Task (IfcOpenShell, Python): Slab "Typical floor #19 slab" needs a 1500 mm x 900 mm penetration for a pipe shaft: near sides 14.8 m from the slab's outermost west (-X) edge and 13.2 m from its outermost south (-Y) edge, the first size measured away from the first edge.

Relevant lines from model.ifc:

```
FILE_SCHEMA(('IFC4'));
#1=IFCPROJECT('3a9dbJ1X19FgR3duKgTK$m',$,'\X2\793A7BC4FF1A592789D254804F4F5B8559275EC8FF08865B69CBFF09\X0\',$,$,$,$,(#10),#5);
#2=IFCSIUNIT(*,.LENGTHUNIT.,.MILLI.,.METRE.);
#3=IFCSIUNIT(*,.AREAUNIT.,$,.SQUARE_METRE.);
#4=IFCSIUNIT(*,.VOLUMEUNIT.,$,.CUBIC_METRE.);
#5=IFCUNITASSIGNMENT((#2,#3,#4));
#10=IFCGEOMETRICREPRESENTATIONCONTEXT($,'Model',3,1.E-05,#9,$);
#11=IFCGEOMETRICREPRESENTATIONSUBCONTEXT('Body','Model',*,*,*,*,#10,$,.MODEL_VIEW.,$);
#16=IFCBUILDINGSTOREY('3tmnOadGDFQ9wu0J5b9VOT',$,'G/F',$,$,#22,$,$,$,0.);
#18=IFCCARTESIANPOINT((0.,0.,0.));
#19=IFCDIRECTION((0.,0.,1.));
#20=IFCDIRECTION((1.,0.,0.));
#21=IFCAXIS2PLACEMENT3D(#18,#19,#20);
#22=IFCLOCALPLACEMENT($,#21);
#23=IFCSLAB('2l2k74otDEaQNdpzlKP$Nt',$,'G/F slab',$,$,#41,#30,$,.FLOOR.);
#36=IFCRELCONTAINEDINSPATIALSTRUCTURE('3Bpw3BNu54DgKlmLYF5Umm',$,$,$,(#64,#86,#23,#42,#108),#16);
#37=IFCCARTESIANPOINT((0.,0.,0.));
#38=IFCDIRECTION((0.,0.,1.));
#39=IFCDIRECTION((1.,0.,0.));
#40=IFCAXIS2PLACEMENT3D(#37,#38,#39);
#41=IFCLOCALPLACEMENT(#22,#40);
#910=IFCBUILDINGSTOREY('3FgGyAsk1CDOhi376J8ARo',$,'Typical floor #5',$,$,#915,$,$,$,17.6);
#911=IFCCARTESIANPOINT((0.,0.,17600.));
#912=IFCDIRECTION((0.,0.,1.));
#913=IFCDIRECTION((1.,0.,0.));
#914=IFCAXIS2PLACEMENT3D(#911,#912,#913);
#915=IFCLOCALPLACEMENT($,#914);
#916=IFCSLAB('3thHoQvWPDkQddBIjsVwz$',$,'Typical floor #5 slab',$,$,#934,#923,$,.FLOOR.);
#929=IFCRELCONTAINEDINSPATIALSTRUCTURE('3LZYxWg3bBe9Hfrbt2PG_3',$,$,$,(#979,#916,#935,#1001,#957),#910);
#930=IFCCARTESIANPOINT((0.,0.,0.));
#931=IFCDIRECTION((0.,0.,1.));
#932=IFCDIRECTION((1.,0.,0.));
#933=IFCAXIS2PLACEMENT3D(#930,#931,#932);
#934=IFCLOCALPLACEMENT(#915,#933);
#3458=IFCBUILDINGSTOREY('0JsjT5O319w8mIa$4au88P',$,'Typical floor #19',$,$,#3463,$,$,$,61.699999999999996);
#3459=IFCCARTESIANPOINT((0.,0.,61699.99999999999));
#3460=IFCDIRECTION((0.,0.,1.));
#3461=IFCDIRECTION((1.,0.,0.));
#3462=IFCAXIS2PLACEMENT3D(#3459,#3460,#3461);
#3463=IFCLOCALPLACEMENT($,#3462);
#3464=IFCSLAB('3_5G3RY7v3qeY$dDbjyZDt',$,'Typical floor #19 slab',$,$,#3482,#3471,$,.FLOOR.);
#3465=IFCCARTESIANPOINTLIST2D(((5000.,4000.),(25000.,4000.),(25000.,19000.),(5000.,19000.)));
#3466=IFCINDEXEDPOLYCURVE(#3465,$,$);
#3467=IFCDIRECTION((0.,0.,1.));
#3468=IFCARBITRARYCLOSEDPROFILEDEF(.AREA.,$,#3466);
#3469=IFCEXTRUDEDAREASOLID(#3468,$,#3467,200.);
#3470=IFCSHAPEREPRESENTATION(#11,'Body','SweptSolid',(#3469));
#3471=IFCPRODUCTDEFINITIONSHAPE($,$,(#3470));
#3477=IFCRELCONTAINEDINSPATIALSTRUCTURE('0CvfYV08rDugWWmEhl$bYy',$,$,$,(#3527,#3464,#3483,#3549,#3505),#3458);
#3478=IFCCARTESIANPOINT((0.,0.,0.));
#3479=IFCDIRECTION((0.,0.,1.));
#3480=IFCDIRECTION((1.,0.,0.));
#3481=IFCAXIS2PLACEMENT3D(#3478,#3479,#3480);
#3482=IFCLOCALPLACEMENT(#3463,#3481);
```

```python
import numpy as np
import ifcopenshell
import ifcopenshell.api.feature
import ifcopenshell.api.geometry
import ifcopenshell.api.root
import ifcopenshell.geom
import ifcopenshell.util.placement
import ifcopenshell.util.representation
import ifcopenshell.util.shape
import ifcopenshell.util.unit

model = ifcopenshell.open("model.ifc")
unit_scale = ifcopenshell.util.unit.calculate_unit_scale(model)
settings = ifcopenshell.geom.settings()


def volume(element):
    """Net volume in cubic metres, openings subtracted."""
    shape = ifcopenshell.geom.create_shape(settings, element)
    return ifcopenshell.util.shape.get_volume(shape.geometry)


slab = model.by_guid("3_5G3RY7v3qeY$dDbjyZDt")
before = volume(slab)

# Extent in the slab's own axes, in metres. The edges named are its -X and -Y sides.
slab_shape = ifcopenshell.geom.create_shape(settings, slab)
vertices = ifcopenshell.util.shape.get_vertices(slab_shape.geometry)
x_min, y_min, bottom = vertices.min(axis=0)
top = vertices[:, 2].max()

opening = ifcopenshell.api.root.create_entity(model, ifc_class="IfcOpeningElement", name="Pipe shaft opening", predefined_type="OPENING")
context = ifcopenshell.util.representation.get_context(model, "Model", "Body", "MODEL_VIEW")
width, depth = 1.5, 0.9
outline = [(0.0, 0.0), (width, 0.0), (width, depth), (0.0, depth), (0.0, 0.0)]
# Overshoot both faces by 50 mm so the cut is clean.
shape = ifcopenshell.api.geometry.add_slab_representation(
    model, context=context, depth=top - bottom + 0.1, polyline=outline
)
ifcopenshell.api.geometry.assign_representation(model, product=opening, representation=shape)

matrix = ifcopenshell.util.placement.get_local_placement(slab.ObjectPlacement)
matrix[:, 3] = matrix @ np.append(np.array([x_min + 14.8, y_min + 13.2, bottom - 0.05]) / unit_scale, 1.0)
ifcopenshell.api.geometry.edit_object_placement(model, product=opening, matrix=matrix, is_si=False)
ifcopenshell.api.feature.add_feature(model, feature=opening, element=slab)

after = volume(slab)

print(f"slab volume {before:.3f} -> {after:.3f} m3")

model.write("model_v2.ifc")
```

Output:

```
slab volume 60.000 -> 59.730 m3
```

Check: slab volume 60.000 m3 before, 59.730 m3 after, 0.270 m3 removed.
